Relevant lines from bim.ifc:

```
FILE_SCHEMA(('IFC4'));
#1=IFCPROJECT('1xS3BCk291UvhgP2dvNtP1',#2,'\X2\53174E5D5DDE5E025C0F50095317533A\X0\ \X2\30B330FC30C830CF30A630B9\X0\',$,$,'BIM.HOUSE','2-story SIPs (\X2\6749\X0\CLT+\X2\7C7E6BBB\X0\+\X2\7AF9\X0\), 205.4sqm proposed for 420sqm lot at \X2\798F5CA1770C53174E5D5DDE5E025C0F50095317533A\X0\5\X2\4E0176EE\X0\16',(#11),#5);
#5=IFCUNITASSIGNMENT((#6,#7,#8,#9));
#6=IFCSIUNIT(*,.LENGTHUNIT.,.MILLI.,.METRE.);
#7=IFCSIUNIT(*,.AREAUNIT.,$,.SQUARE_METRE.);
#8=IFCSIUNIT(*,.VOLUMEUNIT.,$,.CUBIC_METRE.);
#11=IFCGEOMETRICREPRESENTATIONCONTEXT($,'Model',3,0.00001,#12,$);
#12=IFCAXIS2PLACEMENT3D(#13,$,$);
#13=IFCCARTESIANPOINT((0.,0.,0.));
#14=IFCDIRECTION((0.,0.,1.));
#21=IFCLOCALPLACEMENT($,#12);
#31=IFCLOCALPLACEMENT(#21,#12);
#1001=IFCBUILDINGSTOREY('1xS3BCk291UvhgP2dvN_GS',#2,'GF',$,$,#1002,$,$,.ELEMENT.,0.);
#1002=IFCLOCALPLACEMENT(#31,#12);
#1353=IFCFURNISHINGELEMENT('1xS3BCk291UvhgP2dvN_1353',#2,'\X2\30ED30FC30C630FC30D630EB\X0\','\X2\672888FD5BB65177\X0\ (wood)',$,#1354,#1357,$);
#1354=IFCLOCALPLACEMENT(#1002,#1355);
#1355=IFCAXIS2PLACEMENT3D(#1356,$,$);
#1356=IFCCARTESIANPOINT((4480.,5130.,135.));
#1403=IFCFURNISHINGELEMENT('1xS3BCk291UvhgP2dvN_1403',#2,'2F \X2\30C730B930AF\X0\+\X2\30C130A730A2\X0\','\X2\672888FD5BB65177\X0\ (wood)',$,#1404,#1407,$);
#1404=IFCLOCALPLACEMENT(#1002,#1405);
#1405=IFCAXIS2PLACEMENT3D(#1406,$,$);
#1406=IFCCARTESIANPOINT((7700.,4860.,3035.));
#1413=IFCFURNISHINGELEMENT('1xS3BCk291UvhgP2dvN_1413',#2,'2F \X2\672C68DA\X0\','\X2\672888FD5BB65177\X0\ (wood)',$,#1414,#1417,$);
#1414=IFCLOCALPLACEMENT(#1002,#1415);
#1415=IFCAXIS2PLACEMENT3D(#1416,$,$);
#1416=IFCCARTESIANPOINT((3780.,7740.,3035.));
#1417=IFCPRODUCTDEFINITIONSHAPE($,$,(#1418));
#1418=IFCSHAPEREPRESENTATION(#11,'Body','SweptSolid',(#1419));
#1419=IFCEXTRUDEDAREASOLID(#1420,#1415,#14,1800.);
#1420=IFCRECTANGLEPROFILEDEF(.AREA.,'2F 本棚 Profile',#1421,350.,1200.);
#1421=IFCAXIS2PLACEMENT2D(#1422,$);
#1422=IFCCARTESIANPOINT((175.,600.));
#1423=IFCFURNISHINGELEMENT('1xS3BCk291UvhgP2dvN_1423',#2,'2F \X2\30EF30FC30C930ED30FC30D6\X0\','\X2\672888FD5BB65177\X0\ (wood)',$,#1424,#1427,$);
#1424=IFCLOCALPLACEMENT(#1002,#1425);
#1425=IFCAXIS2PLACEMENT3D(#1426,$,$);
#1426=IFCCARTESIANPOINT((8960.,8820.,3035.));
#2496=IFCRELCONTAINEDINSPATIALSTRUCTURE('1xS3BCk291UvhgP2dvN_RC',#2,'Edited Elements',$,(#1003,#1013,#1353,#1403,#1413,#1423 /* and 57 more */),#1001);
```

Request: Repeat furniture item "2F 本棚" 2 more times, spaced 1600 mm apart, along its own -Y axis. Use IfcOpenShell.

```python
import ifcopenshell
import ifcopenshell.api.geometry
import ifcopenshell.api.root
import ifcopenshell.util.element
import ifcopenshell.util.placement

model = ifcopenshell.open("bim.ifc")


def reuse_history(source, copy):
    """copy_class also copies each property set's owner history, people and application; keep the originals."""
    for rel in copy.IsDefinedBy:
        if rel.is_a("IfcRelDefinesByProperties") and (history := rel.RelatingPropertyDefinition.OwnerHistory):
            rel.RelatingPropertyDefinition.OwnerHistory = source.OwnerHistory
            ifcopenshell.util.element.remove_deep2(model, history)


source = model.by_guid("1xS3BCk291UvhgP2dvN_1413")
base = ifcopenshell.util.placement.get_local_placement(source.ObjectPlacement)
step = -base[:3, 1] * 1600.0

for i in range(1, 3):
    copy = ifcopenshell.api.root.copy_class(model, product=source)
    copy.Representation = ifcopenshell.util.element.copy_deep(
        model, source.Representation, exclude=["IfcGeometricRepresentationContext", "IfcRepresentationMap"]
    )
    reuse_history(source, copy)
    matrix = base.copy()
    matrix[:3, 3] += i * step
    print("added at", matrix[:3, 3].round(3) + 0.0)
    ifcopenshell.api.geometry.edit_object_placement(model, product=copy, matrix=matrix, is_si=False)

model.write("bim_rev.ifc")
```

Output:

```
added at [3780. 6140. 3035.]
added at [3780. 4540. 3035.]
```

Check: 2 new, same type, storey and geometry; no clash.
